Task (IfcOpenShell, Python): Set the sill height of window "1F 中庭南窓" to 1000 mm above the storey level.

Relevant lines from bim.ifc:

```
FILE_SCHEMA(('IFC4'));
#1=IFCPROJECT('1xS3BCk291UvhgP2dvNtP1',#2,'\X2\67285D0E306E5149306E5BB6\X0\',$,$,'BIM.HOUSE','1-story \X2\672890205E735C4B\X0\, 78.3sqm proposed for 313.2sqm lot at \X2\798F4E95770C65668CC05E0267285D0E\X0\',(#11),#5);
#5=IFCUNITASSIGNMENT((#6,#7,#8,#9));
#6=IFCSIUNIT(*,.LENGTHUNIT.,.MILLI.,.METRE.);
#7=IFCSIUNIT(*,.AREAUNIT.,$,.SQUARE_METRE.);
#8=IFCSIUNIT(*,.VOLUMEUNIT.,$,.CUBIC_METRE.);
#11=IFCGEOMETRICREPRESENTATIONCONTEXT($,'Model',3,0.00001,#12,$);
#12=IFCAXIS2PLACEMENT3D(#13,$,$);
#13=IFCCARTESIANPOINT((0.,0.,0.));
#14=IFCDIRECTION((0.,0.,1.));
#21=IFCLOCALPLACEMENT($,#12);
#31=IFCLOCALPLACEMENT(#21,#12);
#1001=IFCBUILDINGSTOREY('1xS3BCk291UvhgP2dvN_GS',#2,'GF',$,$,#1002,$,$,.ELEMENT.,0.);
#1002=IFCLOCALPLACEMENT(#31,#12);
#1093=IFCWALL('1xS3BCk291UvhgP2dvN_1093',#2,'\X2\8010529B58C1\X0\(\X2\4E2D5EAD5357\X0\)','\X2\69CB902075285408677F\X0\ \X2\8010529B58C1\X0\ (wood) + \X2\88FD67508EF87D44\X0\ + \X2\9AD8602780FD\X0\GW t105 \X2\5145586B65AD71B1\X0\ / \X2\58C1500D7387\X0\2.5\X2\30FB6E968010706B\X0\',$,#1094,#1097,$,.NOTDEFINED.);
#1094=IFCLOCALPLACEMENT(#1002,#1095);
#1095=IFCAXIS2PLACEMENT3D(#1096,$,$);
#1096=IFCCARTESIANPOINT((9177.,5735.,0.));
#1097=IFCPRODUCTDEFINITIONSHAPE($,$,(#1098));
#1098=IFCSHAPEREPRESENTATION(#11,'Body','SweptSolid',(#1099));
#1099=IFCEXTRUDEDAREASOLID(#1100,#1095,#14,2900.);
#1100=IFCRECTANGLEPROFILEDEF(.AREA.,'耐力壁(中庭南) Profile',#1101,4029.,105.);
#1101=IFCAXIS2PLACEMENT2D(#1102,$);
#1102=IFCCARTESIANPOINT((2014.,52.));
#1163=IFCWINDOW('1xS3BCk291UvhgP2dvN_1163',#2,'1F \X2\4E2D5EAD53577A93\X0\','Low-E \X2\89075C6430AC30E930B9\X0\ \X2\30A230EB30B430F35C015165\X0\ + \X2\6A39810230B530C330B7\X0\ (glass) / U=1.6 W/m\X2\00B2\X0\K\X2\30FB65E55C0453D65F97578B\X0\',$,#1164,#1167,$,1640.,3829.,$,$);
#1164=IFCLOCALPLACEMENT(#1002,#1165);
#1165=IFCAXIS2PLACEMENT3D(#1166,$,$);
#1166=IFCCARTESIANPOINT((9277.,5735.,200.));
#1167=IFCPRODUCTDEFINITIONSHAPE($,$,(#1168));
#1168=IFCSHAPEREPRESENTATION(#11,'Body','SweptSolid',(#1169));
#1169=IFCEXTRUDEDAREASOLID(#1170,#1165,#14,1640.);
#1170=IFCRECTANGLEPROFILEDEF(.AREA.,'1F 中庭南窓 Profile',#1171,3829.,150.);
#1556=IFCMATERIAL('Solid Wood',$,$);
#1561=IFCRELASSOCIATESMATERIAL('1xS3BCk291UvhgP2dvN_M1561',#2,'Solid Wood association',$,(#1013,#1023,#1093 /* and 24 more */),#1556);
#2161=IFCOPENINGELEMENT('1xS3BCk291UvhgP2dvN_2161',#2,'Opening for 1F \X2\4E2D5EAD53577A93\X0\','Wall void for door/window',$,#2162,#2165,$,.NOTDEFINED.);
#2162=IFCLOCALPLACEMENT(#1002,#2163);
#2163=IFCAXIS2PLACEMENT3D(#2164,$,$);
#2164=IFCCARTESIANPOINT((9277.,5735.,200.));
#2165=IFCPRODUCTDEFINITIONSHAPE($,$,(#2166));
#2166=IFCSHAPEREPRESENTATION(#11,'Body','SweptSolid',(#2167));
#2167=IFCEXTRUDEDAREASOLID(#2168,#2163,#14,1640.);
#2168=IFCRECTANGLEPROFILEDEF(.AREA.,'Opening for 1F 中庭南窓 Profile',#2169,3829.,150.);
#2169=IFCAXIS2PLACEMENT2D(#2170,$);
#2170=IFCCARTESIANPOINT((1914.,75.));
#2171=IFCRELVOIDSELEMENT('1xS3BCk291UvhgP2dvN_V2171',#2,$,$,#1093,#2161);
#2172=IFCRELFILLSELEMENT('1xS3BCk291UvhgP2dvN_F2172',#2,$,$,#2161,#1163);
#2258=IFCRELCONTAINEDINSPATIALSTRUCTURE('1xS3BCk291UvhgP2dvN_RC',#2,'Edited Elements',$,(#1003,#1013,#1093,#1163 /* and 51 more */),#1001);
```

```python
import numpy as np
import ifcopenshell
import ifcopenshell.api.geometry
import ifcopenshell.geom
import ifcopenshell.util.element
import ifcopenshell.util.placement
import ifcopenshell.util.shape
import ifcopenshell.util.unit

model = ifcopenshell.open("bim.ifc")
unit_scale = ifcopenshell.util.unit.calculate_unit_scale(model)

window = model.by_id(1163)
opening = window.FillsVoids[0].RelatingOpeningElement
storey = ifcopenshell.util.element.get_container(window, ifc_class="IfcBuildingStorey")
level = ifcopenshell.util.placement.get_local_placement(storey.ObjectPlacement)[2, 3]

# The opening's origin need not be at the sill, so measure its lowest point.
shape = ifcopenshell.geom.create_shape(ifcopenshell.geom.settings(), opening)
bottom = ifcopenshell.util.shape.get_shape_bottom_elevation(shape, shape.geometry) / unit_scale
dz = level + 1 / unit_scale - bottom

shift = np.array([0.0, 0.0, dz])
# The window is not placed relative to its opening, so move both.
for product in (opening, window):
    matrix = ifcopenshell.util.placement.get_local_placement(product.ObjectPlacement)
    matrix[:3, 3] += shift
    ifcopenshell.api.geometry.edit_object_placement(model, product=product, matrix=matrix, is_si=False)

print(f"moved by {dz * unit_scale:+.3f} m")

model.write("bim-out.ifc")
```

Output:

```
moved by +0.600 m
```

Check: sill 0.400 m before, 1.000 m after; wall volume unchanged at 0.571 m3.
